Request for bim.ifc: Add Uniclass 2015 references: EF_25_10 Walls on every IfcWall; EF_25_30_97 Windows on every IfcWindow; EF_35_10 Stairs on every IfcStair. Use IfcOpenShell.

First a look at what the model holds.

```python
import ifcopenshell

model = ifcopenshell.open("bim.ifc")
print(model.schema)
print("classifications:", [c.Name for c in model.by_type("IfcClassification")])
for ifc_class in ("IfcDoor", "IfcRoof", "IfcStair", "IfcWall", "IfcWindow"):
    print(ifc_class, len(model.by_type(ifc_class)))
```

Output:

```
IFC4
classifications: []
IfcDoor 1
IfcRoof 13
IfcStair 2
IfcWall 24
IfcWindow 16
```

```python
import ifcopenshell
import ifcopenshell.api.classification

model = ifcopenshell.open("bim.ifc")

system = ifcopenshell.api.classification.add_classification(model, classification="Uniclass 2015")

codes = {
    "IfcWall": ("EF_25_10", "Walls"),
    "IfcWindow": ("EF_25_30_97", "Windows"),
    "IfcStair": ("EF_35_10", "Stairs"),
}
for ifc_class, (code, name) in codes.items():
    products = model.by_type(ifc_class)
    ifcopenshell.api.classification.add_reference(
        model, products=products, classification=system, identification=code, name=name
    )
    print(code, len(products))

model.write("bim_rev.ifc")
```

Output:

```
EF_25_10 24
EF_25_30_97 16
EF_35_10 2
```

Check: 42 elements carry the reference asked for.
